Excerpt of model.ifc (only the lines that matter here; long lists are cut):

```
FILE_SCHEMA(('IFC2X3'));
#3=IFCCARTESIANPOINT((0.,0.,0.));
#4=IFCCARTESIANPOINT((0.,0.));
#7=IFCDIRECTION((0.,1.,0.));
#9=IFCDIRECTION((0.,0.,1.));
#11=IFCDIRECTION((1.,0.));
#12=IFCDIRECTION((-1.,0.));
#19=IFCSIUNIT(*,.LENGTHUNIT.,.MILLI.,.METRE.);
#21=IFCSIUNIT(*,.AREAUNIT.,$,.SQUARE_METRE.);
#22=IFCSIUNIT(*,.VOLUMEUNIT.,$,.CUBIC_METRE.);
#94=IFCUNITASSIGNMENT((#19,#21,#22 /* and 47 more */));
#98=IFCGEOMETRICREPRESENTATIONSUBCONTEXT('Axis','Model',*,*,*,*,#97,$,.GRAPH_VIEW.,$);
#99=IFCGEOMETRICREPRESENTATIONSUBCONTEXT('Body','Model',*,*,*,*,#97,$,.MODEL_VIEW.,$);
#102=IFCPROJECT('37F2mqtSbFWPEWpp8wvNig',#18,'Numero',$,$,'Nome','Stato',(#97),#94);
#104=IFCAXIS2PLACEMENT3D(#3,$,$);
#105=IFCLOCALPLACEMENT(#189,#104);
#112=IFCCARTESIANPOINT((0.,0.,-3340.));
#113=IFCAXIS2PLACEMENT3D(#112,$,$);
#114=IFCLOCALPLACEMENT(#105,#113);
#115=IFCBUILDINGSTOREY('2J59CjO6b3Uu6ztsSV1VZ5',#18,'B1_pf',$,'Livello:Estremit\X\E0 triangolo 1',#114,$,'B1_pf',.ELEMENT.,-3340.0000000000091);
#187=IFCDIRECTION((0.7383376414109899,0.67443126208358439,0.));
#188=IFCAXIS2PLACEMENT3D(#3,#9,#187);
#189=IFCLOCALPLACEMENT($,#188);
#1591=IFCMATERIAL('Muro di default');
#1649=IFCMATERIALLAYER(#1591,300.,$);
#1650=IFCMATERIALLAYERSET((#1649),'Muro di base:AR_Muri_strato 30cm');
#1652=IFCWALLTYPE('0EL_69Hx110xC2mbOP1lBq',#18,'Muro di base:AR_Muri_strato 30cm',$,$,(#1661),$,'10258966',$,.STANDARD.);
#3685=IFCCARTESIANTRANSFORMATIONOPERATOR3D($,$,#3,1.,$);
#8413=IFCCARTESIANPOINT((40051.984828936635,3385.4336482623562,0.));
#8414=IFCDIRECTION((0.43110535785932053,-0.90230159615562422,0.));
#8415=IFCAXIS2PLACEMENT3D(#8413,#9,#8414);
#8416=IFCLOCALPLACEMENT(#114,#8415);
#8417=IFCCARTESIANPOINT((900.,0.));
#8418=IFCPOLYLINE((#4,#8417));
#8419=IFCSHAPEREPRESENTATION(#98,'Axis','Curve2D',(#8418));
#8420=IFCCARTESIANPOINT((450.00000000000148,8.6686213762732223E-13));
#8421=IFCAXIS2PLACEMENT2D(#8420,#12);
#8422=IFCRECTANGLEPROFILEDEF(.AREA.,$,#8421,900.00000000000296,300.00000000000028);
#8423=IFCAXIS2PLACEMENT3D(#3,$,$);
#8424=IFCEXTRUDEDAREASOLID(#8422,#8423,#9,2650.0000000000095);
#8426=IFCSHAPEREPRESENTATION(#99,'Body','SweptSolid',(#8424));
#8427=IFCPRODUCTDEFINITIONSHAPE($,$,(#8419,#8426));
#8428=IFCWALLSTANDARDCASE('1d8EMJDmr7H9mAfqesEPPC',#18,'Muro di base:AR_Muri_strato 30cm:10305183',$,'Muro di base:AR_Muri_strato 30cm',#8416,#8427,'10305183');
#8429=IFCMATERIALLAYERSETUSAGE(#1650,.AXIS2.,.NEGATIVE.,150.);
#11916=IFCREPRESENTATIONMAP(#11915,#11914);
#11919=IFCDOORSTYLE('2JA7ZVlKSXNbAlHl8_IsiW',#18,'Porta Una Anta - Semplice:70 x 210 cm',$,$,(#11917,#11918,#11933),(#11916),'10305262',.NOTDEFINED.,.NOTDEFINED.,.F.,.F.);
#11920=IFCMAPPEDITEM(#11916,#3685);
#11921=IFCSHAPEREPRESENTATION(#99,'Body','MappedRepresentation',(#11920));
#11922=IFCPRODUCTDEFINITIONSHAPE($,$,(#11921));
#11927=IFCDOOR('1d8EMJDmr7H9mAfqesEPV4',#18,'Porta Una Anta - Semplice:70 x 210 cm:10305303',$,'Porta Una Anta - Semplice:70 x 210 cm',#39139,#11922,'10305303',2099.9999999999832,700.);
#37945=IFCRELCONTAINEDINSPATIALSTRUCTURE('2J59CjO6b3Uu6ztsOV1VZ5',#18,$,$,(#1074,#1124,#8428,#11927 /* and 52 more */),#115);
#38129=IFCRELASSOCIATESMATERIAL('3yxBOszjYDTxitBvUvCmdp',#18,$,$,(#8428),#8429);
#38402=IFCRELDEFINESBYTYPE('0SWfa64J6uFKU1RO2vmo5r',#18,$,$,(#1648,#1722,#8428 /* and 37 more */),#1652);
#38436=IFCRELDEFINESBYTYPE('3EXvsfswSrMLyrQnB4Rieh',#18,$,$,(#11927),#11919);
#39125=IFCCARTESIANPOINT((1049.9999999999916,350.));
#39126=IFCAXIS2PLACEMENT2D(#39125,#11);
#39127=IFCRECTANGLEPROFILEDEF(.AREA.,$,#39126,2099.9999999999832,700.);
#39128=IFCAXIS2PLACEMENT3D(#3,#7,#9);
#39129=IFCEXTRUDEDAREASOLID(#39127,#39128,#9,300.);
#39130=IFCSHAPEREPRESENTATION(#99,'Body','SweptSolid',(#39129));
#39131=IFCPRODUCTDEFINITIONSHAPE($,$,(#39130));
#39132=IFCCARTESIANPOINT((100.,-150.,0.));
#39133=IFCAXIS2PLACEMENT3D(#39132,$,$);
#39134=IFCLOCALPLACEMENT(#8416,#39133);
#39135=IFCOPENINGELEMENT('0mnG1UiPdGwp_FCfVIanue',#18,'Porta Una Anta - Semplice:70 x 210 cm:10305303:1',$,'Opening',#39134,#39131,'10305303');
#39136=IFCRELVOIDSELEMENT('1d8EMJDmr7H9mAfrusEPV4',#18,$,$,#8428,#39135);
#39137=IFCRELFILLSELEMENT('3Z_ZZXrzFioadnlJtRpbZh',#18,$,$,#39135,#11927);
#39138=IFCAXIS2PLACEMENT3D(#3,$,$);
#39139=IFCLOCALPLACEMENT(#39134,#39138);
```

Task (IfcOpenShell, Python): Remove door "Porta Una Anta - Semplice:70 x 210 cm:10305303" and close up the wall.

```python
import ifcopenshell
import ifcopenshell.api.feature
import ifcopenshell.api.root
import ifcopenshell.geom
import ifcopenshell.util.shape

model = ifcopenshell.open("model.ifc")
settings = ifcopenshell.geom.settings()


def volume(element):
    """Net volume in cubic metres, openings subtracted."""
    shape = ifcopenshell.geom.create_shape(settings, element)
    return ifcopenshell.util.shape.get_volume(shape.geometry)


door = model.by_guid("1d8EMJDmr7H9mAfqesEPV4")
opening = door.FillsVoids[0].RelatingOpeningElement
wall = opening.VoidsElements[0].RelatingBuildingElement
before = volume(wall)

ifcopenshell.api.root.remove_product(model, product=door)
ifcopenshell.api.feature.remove_feature(model, feature=opening)

after = volume(wall)

print(f"wall volume {before:.3f} -> {after:.3f} m3")

model.write("model-out.ifc")
```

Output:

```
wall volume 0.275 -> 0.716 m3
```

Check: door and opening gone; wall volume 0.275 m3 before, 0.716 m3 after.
